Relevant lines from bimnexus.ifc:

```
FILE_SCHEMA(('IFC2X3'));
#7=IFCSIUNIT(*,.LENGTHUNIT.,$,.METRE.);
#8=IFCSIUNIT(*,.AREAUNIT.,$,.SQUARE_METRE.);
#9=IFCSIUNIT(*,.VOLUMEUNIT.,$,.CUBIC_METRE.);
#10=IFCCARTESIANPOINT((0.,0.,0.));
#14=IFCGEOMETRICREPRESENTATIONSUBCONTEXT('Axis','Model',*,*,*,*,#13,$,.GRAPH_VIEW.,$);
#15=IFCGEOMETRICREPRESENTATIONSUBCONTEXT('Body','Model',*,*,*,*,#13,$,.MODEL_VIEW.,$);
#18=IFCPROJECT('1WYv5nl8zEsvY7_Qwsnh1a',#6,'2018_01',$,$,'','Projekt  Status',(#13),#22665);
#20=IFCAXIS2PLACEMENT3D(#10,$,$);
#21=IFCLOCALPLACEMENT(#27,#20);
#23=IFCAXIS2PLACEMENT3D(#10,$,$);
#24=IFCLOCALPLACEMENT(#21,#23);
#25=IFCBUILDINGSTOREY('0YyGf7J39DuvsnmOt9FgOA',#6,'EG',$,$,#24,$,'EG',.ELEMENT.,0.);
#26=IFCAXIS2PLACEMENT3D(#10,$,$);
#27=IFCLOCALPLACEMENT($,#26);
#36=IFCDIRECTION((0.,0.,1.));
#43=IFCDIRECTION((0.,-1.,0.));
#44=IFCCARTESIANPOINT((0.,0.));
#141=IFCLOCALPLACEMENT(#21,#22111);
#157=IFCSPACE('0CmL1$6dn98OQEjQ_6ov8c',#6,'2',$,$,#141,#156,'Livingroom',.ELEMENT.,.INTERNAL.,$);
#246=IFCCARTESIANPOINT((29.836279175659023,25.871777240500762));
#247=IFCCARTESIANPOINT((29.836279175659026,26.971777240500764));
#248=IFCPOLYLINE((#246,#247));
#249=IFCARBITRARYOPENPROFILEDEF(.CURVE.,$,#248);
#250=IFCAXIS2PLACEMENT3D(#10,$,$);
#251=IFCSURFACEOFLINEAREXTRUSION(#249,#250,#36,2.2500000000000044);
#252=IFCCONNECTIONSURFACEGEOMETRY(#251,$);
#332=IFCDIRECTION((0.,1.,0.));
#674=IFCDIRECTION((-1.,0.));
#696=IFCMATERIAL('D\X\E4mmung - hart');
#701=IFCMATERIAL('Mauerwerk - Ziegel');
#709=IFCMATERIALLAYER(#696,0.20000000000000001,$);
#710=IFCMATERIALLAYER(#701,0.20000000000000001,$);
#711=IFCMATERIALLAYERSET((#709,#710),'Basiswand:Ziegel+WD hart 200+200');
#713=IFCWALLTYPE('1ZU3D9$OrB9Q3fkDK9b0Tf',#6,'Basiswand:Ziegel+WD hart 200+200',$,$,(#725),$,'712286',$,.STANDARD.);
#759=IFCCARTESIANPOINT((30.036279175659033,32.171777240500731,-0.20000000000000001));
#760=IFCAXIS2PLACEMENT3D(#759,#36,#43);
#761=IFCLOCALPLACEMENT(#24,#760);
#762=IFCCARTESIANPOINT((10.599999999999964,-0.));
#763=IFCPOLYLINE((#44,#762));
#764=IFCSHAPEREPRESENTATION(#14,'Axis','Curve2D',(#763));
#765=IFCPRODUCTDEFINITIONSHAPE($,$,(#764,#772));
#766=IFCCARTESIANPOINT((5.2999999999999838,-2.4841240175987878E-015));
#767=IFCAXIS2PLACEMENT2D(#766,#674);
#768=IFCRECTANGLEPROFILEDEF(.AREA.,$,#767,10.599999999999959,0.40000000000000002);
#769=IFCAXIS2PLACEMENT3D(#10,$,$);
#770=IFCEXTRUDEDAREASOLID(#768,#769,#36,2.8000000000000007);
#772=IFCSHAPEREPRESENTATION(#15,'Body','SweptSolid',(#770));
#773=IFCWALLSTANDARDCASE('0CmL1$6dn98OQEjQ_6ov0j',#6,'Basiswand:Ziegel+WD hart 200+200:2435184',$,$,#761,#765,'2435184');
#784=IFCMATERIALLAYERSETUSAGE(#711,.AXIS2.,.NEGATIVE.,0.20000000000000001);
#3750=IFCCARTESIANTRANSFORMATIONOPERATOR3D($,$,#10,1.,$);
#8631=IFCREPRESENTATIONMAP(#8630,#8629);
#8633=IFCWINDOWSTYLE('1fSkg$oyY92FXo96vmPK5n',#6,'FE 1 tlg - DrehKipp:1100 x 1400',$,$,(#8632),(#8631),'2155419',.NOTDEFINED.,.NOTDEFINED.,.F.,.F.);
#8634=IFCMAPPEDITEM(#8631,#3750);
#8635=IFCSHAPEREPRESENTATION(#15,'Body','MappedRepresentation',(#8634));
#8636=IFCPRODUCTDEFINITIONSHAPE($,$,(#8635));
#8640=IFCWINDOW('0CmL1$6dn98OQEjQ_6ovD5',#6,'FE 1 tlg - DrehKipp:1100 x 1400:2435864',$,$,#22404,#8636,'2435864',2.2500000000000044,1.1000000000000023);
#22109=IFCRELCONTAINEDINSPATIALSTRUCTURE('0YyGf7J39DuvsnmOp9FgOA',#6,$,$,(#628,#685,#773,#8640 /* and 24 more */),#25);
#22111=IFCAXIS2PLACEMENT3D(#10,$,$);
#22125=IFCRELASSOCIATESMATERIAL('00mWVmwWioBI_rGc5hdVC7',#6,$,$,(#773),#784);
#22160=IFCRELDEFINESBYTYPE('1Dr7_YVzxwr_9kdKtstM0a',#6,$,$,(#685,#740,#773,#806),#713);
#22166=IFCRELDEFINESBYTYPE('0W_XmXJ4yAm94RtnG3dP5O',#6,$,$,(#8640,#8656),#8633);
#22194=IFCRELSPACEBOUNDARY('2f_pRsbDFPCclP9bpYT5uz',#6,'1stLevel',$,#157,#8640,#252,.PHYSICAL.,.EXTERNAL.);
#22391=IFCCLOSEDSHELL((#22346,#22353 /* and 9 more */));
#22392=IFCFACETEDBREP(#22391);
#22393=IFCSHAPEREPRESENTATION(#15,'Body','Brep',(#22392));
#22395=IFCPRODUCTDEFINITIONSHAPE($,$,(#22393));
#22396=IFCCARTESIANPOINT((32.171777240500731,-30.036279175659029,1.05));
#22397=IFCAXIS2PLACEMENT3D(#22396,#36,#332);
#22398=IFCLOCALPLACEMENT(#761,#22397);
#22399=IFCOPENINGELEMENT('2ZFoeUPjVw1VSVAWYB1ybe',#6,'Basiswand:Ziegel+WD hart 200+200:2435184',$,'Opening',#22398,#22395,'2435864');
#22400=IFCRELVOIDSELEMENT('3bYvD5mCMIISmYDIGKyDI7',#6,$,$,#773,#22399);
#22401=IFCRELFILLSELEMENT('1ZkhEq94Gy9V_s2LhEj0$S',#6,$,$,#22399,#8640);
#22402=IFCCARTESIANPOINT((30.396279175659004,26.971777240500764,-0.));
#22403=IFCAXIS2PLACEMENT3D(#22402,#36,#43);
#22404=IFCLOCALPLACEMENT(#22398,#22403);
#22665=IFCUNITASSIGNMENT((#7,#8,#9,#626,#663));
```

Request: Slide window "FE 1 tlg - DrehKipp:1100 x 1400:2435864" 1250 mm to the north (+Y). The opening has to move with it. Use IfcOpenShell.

```python
import numpy as np
import ifcopenshell
import ifcopenshell.api.geometry
import ifcopenshell.util.placement
import ifcopenshell.util.unit

model = ifcopenshell.open("bimnexus.ifc")
unit_scale = ifcopenshell.util.unit.calculate_unit_scale(model)

window = model.by_guid("0CmL1$6dn98OQEjQ_6ovD5")
opening = window.FillsVoids[0].RelatingOpeningElement
wall = opening.VoidsElements[0].RelatingBuildingElement

wall_matrix = ifcopenshell.util.placement.get_local_placement(wall.ObjectPlacement)
shift = wall_matrix[:3, 0] * -1.25 / unit_scale
before = ifcopenshell.util.placement.get_local_placement(window.ObjectPlacement)[:3, 3].copy()

# The window is placed relative to its opening, so it follows when the opening moves.
matrix = ifcopenshell.util.placement.get_local_placement(opening.ObjectPlacement)
matrix[:3, 3] += shift
ifcopenshell.api.geometry.edit_object_placement(
    model, product=opening, matrix=matrix, is_si=False, should_transform_children=True
)

# Space boundary surfaces are stored in each space's coordinates; move them too.
for rel in window.ProvidesBoundaries:
    if not rel.ConnectionGeometry:
        continue
    surface = rel.ConnectionGeometry.SurfaceOnRelatingElement
    space_matrix = ifcopenshell.util.placement.get_local_placement(rel.RelatingSpace.ObjectPlacement)
    point = np.array(surface.Position.Location.Coordinates) + space_matrix[:3, :3].T @ shift
    surface.Position = model.createIfcAxis2Placement3D(
        model.createIfcCartesianPoint(point.tolist()), surface.Position.Axis, surface.Position.RefDirection
    )

after = ifcopenshell.util.placement.get_local_placement(window.ObjectPlacement)[:3, 3]
print("window moved by", (after - before).round(3) + 0.0)

model.write("bimnexus_rev.ifc")
```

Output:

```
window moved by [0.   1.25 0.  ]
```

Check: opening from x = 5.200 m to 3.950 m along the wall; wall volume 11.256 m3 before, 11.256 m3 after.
